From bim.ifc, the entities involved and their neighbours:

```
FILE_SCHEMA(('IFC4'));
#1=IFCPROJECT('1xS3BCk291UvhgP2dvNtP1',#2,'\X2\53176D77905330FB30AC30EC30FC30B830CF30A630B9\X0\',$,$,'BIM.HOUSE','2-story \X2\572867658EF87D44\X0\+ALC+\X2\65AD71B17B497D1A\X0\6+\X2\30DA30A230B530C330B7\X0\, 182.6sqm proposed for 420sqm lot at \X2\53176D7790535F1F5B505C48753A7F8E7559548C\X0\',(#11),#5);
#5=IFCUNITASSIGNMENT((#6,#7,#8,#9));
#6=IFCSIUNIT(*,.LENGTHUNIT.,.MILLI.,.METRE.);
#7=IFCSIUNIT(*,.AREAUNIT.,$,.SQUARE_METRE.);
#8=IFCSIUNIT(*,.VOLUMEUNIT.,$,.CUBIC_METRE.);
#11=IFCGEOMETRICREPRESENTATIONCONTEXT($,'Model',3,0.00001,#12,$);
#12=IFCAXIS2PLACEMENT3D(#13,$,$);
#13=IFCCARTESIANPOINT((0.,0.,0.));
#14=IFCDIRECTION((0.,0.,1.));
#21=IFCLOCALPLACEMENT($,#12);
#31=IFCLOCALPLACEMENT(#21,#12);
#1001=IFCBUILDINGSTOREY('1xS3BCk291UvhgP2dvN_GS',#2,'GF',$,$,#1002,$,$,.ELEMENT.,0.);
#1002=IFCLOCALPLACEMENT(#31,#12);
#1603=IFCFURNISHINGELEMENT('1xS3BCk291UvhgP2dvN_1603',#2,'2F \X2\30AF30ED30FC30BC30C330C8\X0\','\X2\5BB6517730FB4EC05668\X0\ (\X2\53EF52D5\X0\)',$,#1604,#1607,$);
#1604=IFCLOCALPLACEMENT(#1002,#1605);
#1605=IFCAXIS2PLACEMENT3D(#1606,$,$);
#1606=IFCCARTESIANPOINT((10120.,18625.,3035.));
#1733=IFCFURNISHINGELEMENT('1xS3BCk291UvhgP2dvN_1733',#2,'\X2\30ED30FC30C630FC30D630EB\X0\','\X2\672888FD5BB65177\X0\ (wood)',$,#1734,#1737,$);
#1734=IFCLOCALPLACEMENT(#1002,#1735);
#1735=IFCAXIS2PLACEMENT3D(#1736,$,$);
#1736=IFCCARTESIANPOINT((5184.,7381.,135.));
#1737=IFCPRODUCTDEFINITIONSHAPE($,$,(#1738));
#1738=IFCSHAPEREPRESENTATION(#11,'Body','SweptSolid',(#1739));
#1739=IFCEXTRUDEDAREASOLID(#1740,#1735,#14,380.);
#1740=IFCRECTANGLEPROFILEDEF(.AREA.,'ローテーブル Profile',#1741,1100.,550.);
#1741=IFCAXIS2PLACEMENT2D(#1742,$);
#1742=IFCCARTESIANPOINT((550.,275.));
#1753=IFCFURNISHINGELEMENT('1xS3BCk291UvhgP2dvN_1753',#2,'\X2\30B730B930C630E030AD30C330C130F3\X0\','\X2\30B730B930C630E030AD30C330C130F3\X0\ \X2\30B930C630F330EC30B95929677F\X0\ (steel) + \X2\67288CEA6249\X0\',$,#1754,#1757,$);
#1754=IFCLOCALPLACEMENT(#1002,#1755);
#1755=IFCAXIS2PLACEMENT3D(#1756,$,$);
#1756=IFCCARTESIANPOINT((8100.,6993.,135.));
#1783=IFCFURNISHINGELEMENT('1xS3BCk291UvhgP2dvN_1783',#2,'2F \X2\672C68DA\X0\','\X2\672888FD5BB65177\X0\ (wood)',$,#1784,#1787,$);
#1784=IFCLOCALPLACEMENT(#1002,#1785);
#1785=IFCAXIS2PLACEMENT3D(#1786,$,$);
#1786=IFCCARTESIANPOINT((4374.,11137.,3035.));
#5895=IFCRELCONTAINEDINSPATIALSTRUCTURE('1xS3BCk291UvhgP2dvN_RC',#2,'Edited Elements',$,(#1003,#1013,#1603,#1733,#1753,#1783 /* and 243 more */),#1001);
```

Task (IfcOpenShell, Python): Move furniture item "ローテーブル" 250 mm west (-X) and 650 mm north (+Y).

```python
import ifcopenshell
import ifcopenshell.api.geometry
import ifcopenshell.util.placement
import ifcopenshell.util.unit

model = ifcopenshell.open("bim.ifc")
unit_scale = ifcopenshell.util.unit.calculate_unit_scale(model)

item = model.by_id(1733)
matrix = ifcopenshell.util.placement.get_local_placement(item.ObjectPlacement)
matrix[0, 3] -= 0.25 / unit_scale
matrix[1, 3] += 0.65 / unit_scale
ifcopenshell.api.geometry.edit_object_placement(model, product=item, matrix=matrix, is_si=False)

print(ifcopenshell.util.placement.get_local_placement(item.ObjectPlacement).round(3) + 0.0)

model.write("bim_v2.ifc")
```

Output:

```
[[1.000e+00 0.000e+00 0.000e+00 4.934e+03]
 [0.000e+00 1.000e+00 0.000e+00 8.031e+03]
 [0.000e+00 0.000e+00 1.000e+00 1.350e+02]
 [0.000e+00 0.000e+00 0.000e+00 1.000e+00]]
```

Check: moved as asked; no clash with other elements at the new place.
